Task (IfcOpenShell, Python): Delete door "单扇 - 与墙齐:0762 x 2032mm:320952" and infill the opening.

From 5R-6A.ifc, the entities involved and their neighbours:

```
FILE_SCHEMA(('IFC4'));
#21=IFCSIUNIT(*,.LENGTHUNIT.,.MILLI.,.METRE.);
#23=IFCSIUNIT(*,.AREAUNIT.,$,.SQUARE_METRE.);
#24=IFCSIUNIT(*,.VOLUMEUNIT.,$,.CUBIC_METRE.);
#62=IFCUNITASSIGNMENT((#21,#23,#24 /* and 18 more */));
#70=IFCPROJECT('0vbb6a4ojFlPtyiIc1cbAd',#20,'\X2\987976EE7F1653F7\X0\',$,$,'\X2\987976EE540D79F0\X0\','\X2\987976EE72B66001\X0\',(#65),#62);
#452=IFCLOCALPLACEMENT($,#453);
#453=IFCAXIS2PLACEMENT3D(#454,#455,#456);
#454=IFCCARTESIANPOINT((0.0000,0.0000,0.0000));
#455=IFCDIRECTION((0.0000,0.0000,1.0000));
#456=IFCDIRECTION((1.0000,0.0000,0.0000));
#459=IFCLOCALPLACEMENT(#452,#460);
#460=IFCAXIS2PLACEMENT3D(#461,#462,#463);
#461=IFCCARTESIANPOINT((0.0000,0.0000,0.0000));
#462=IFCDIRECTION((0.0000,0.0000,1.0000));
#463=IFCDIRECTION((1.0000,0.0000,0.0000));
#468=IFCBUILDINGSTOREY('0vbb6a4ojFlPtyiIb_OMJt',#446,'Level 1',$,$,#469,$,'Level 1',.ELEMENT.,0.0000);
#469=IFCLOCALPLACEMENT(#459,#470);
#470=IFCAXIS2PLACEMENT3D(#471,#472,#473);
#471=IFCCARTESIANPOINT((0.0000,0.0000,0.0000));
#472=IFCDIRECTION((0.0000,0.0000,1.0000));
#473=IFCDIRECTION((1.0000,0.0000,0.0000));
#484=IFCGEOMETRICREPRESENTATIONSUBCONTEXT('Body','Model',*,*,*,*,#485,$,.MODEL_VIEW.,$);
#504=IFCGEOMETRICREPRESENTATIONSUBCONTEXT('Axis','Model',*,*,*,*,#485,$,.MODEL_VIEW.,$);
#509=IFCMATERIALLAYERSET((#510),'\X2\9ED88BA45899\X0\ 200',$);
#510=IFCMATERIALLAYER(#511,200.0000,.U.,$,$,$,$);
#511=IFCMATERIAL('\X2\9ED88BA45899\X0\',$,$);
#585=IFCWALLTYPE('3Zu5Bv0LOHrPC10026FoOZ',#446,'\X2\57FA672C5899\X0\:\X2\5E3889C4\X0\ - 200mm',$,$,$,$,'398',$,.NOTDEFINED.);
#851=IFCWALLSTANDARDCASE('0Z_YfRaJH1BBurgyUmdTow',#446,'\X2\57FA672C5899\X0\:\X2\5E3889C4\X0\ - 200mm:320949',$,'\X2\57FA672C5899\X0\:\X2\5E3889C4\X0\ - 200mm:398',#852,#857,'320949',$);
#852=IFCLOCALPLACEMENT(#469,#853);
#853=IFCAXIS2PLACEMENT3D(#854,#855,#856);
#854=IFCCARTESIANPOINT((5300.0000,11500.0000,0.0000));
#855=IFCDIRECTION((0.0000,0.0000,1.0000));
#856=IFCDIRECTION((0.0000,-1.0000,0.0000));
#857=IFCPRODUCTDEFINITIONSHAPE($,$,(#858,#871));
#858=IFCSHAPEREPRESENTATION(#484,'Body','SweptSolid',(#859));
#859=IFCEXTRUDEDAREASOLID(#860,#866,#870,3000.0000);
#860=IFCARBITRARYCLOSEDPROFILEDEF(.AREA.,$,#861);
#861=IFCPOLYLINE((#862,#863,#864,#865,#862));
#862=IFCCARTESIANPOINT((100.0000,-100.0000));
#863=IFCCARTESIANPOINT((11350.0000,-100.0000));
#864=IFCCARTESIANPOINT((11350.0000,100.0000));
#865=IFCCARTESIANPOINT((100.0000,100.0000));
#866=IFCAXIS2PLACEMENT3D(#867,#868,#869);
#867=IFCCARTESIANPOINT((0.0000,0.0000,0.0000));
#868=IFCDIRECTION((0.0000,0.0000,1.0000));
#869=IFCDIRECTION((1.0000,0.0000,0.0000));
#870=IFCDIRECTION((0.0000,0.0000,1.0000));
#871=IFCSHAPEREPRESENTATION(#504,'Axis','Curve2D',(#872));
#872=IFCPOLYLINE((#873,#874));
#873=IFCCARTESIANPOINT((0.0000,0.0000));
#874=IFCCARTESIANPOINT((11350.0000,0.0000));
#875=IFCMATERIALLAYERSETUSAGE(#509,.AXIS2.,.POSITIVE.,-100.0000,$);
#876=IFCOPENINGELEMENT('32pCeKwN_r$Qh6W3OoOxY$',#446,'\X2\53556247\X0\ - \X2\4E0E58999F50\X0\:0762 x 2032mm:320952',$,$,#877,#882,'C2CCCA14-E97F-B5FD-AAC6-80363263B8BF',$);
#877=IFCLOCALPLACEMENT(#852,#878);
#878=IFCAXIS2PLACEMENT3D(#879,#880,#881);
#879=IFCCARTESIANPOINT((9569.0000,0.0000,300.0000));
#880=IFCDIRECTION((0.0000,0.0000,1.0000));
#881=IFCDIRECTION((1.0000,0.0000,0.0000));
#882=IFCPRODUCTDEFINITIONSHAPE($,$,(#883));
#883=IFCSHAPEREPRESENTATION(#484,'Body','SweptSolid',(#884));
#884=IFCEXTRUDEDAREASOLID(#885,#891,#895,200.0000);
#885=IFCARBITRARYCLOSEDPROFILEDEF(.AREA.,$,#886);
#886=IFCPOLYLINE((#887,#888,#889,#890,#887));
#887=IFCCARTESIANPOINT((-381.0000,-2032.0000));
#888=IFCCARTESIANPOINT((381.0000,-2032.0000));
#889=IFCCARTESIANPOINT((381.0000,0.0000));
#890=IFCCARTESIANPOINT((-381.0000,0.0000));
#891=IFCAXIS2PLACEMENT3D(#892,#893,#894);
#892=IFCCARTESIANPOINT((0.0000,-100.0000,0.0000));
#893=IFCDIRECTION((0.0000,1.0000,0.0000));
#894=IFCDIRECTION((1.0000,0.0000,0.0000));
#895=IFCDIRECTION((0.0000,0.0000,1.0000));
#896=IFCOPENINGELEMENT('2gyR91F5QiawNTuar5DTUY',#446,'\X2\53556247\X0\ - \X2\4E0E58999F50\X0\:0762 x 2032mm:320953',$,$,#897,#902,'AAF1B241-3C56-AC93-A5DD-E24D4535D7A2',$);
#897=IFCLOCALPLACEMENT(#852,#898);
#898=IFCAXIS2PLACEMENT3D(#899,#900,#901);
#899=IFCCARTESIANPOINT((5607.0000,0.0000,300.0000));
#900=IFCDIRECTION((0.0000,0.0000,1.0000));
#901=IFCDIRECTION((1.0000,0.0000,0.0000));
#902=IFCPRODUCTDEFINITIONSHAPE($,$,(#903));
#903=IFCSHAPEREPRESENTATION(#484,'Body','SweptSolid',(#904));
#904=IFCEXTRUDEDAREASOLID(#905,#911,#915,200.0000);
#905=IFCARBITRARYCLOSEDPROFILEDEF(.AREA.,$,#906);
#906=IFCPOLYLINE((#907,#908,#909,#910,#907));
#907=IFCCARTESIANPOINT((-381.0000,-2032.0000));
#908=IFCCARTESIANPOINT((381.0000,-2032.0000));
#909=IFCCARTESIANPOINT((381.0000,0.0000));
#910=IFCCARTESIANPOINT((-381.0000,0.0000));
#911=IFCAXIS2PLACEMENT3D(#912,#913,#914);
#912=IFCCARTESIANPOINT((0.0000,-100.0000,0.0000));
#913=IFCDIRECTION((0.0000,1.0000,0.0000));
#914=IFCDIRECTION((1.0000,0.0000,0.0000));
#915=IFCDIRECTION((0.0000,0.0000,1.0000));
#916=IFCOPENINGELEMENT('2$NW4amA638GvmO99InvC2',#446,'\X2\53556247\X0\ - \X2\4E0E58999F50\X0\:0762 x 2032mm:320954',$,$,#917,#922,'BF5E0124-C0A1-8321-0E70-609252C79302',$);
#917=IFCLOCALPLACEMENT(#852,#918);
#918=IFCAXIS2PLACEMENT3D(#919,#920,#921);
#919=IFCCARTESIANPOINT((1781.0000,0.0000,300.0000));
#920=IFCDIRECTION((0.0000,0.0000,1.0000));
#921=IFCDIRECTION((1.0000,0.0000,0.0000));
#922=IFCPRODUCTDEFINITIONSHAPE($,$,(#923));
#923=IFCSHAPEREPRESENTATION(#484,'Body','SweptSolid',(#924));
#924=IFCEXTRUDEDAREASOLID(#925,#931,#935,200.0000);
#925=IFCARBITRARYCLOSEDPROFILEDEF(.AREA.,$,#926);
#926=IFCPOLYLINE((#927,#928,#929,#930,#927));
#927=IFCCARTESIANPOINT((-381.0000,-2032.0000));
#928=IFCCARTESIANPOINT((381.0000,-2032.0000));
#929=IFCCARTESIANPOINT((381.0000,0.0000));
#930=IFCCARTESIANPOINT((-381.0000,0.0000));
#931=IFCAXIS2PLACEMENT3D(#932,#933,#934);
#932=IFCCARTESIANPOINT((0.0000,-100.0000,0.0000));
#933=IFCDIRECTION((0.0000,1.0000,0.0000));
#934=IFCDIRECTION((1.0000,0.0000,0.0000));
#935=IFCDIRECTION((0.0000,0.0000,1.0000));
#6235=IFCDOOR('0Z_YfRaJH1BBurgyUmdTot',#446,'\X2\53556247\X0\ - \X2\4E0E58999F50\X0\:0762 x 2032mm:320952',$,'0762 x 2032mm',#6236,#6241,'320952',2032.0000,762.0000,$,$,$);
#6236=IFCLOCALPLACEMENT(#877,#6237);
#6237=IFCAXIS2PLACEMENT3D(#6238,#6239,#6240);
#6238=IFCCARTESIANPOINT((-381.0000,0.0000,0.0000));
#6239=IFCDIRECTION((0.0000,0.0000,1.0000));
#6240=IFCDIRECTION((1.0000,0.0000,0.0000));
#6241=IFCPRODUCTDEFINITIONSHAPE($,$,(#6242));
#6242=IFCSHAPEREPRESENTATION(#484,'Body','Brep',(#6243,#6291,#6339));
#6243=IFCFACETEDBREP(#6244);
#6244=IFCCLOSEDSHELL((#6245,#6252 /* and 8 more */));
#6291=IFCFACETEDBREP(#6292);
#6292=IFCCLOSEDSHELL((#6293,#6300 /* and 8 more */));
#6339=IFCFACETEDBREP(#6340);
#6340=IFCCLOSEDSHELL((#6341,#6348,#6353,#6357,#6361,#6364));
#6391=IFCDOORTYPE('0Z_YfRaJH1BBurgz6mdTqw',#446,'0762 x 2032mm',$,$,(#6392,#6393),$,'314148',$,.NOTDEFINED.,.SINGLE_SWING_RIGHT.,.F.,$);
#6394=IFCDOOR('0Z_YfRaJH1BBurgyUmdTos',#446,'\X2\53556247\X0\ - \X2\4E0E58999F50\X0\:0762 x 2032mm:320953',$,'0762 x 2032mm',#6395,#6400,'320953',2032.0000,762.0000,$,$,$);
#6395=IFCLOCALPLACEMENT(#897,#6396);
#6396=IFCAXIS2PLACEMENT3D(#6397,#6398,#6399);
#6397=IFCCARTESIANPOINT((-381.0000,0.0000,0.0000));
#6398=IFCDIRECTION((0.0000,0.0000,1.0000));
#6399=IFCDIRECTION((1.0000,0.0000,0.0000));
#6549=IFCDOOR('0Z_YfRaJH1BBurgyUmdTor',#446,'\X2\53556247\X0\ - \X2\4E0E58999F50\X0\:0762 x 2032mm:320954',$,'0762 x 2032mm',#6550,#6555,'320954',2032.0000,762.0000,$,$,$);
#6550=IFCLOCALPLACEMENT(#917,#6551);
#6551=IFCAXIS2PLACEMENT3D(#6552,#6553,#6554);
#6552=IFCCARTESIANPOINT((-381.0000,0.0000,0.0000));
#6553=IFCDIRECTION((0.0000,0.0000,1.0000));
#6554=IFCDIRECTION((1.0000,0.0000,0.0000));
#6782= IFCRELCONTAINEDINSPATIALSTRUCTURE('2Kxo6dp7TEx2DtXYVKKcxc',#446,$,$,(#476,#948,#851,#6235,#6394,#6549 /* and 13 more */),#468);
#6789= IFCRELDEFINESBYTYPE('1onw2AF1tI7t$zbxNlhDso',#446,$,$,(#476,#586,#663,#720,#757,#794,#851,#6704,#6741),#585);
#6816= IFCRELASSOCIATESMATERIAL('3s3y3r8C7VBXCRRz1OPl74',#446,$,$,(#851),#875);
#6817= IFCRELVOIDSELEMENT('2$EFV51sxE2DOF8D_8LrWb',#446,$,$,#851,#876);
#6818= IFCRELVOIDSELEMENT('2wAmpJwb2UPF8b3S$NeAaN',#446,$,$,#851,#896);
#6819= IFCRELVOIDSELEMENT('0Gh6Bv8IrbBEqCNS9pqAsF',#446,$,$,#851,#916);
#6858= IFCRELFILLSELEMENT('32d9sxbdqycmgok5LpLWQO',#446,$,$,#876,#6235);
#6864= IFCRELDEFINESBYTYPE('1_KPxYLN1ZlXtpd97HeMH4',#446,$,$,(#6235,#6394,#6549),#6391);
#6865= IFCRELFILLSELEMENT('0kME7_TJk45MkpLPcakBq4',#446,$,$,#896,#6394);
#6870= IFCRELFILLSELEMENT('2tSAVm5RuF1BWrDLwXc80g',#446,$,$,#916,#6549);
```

```python
import ifcopenshell
import ifcopenshell.api.feature
import ifcopenshell.api.root
import ifcopenshell.geom
import ifcopenshell.util.shape

model = ifcopenshell.open("5R-6A.ifc")
settings = ifcopenshell.geom.settings()


def volume(element):
    """Net volume in cubic metres, openings subtracted."""
    shape = ifcopenshell.geom.create_shape(settings, element)
    return ifcopenshell.util.shape.get_volume(shape.geometry)


door = model.by_guid("0Z_YfRaJH1BBurgyUmdTot")
opening = door.FillsVoids[0].RelatingOpeningElement
wall = opening.VoidsElements[0].RelatingBuildingElement
before = volume(wall)

ifcopenshell.api.root.remove_product(model, product=door)
ifcopenshell.api.feature.remove_feature(model, feature=opening)

after = volume(wall)

print(f"wall volume {before:.3f} -> {after:.3f} m3")

model.write("5R-6A_rev.ifc")
```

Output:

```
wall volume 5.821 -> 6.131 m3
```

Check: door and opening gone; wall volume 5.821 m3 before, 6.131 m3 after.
